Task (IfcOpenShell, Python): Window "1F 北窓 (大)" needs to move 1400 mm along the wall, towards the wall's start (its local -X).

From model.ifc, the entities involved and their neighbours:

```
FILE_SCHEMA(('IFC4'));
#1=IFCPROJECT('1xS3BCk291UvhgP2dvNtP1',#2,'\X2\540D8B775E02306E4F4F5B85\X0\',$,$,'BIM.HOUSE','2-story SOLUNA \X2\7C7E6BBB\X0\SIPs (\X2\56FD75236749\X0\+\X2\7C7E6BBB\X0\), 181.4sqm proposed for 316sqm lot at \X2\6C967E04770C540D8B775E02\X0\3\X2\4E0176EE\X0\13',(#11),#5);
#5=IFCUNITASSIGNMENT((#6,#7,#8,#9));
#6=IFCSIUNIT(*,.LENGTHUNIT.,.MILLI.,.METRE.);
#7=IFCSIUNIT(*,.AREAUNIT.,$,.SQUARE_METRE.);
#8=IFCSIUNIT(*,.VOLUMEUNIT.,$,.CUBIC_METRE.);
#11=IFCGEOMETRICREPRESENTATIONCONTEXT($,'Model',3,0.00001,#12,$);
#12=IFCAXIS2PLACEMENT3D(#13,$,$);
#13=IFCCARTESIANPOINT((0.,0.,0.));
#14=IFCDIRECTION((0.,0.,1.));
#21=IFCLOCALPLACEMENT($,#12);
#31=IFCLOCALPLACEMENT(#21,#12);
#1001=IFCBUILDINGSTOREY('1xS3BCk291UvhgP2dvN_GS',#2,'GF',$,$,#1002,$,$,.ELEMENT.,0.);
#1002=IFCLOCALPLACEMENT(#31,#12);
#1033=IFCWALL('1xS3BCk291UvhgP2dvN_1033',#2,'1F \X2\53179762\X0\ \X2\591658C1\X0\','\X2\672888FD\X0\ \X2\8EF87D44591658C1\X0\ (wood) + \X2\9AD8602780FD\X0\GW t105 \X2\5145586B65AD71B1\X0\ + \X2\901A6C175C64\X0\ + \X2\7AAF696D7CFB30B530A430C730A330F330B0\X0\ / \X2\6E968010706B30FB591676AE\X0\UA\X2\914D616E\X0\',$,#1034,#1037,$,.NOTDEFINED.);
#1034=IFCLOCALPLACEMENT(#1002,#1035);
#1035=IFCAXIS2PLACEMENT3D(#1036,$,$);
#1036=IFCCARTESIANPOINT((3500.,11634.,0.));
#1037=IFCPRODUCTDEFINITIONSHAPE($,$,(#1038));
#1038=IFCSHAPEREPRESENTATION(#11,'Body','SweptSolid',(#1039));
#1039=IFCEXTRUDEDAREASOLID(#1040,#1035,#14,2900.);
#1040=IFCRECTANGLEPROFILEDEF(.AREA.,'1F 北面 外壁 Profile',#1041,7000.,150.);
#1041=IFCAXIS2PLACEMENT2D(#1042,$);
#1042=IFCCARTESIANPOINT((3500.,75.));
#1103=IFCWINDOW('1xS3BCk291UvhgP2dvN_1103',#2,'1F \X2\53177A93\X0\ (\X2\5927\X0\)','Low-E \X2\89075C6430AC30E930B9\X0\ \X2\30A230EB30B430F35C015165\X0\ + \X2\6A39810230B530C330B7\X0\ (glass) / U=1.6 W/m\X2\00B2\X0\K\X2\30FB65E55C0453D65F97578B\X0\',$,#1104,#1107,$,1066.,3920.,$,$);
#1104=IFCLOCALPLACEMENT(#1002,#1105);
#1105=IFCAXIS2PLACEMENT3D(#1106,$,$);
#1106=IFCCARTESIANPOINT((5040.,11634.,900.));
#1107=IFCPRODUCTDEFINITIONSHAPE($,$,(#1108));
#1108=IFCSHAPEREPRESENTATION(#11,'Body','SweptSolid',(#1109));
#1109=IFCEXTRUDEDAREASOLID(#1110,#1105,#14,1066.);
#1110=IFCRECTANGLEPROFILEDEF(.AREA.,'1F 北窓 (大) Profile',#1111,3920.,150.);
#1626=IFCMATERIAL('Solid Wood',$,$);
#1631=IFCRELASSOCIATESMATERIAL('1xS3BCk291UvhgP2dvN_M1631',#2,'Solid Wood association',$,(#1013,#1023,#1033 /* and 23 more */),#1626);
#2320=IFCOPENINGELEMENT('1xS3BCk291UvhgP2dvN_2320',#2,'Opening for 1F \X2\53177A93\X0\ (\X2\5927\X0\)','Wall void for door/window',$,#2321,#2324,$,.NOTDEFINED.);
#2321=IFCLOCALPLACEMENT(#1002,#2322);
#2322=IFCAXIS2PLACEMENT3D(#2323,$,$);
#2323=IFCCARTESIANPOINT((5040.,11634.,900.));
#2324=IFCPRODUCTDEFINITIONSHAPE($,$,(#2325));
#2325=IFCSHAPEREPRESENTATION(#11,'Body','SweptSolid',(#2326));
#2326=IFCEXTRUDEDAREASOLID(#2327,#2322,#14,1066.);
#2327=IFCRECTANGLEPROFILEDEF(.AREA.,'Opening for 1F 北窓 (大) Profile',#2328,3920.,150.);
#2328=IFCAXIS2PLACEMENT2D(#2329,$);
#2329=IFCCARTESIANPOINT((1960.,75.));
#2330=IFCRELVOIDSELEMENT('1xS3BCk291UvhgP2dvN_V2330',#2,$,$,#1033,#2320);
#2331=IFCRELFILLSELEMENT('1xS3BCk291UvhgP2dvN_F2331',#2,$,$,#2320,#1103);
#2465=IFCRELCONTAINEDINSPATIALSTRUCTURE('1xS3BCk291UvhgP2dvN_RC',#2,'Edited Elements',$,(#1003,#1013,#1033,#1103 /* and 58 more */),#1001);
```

```python
import ifcopenshell
import ifcopenshell.api.geometry
import ifcopenshell.util.placement
import ifcopenshell.util.unit

model = ifcopenshell.open("model.ifc")
unit_scale = ifcopenshell.util.unit.calculate_unit_scale(model)

window = model.by_id(1103)
opening = window.FillsVoids[0].RelatingOpeningElement
wall = opening.VoidsElements[0].RelatingBuildingElement

wall_matrix = ifcopenshell.util.placement.get_local_placement(wall.ObjectPlacement)
shift = wall_matrix[:3, 0] * -1.4 / unit_scale
before = ifcopenshell.util.placement.get_local_placement(window.ObjectPlacement)[:3, 3].copy()

# The window is not placed relative to its opening, so move both.
for product in (opening, window):
    matrix = ifcopenshell.util.placement.get_local_placement(product.ObjectPlacement)
    matrix[:3, 3] += shift
    ifcopenshell.api.geometry.edit_object_placement(model, product=product, matrix=matrix, is_si=False)

after = ifcopenshell.util.placement.get_local_placement(window.ObjectPlacement)[:3, 3]
print("window moved by", (after - before).round(3) + 0.0)

model.write("model-out.ifc")
```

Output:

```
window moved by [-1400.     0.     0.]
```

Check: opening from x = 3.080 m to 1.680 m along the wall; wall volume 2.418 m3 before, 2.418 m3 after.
